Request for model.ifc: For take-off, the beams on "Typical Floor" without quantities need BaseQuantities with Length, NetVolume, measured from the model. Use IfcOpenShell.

First a look at what the model holds.

```python
import ifcopenshell
import ifcopenshell.util.element
import ifcopenshell.util.unit

model = ifcopenshell.open("model.ifc")
print(model.schema)
for unit_type in ("LENGTHUNIT", "AREAUNIT", "VOLUMEUNIT"):
    print(unit_type, ifcopenshell.util.unit.calculate_unit_scale(model, unit_type))
storey = next(s for s in model.by_type("IfcBuildingStorey") if s.Name == "Typical Floor")
beams = [e for e in ifcopenshell.util.element.get_decomposition(storey) if e.is_a("IfcBeam")]
for e in sorted(beams, key=lambda e: e.id()):
    print(e.id(), e.is_a(), e.Name, list(ifcopenshell.util.element.get_psets(e, qtos_only=True)), sep=" | ")
```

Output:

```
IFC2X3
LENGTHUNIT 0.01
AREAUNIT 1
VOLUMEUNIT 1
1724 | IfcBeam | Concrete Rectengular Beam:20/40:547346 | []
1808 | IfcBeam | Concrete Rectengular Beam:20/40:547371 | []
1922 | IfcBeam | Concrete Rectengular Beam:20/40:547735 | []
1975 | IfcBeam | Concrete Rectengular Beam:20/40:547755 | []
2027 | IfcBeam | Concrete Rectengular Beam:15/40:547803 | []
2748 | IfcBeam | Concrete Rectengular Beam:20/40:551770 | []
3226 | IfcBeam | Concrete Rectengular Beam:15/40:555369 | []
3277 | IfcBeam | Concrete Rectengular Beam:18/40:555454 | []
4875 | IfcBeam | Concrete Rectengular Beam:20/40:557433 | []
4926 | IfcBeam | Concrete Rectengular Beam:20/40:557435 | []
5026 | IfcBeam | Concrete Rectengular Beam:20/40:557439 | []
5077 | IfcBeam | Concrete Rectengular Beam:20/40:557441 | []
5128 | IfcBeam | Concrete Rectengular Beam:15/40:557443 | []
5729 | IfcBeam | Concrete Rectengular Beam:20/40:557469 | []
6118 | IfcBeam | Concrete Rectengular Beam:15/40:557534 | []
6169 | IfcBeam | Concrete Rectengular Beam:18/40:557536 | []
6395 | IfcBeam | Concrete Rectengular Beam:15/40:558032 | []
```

```python
import ifcopenshell
import ifcopenshell.api.pset
import ifcopenshell.geom
import ifcopenshell.util.element
import ifcopenshell.util.shape
import ifcopenshell.util.unit

model = ifcopenshell.open("model.ifc")
unit_scale = ifcopenshell.util.unit.calculate_unit_scale(model)
volume_scale = ifcopenshell.util.unit.calculate_unit_scale(model, "VOLUMEUNIT")
settings = ifcopenshell.geom.settings()

storey = next(s for s in model.by_type("IfcBuildingStorey") if s.Name == "Typical Floor")
beams = [e for e in ifcopenshell.util.element.get_decomposition(storey) if e.is_a("IfcBeam")]

for e in sorted(beams, key=lambda e: e.id()):
    if ifcopenshell.util.element.get_psets(e, qtos_only=True, should_inherit=False):
        continue
    # Geometry comes back in metres, in the element's own axes.
    shape = ifcopenshell.geom.create_shape(settings, e)
    values = {
        "Length": ifcopenshell.util.shape.get_max_xyz(shape.geometry) / unit_scale,
        "NetVolume": ifcopenshell.util.shape.get_volume(shape.geometry) / volume_scale,
    }
    qto = ifcopenshell.api.pset.add_qto(model, product=e, name="BaseQuantities")
    ifcopenshell.api.pset.edit_qto(model, qto=qto, properties=values)
    print(e.id(), {k: round(v, 3) for k, v in values.items()})

model.write("model_edited.ifc")
```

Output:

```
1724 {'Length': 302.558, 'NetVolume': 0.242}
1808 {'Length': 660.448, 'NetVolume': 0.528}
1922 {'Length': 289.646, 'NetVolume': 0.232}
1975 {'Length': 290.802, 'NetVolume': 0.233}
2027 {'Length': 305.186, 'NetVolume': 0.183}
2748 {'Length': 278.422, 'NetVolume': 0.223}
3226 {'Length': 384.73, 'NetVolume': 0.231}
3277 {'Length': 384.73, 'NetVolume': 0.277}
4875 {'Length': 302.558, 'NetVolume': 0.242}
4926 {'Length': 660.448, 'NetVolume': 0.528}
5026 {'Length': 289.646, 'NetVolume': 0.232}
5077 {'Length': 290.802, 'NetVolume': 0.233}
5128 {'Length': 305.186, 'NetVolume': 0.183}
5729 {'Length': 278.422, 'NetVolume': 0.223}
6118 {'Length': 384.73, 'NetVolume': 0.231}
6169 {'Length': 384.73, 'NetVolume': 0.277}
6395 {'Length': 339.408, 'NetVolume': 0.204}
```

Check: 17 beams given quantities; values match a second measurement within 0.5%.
